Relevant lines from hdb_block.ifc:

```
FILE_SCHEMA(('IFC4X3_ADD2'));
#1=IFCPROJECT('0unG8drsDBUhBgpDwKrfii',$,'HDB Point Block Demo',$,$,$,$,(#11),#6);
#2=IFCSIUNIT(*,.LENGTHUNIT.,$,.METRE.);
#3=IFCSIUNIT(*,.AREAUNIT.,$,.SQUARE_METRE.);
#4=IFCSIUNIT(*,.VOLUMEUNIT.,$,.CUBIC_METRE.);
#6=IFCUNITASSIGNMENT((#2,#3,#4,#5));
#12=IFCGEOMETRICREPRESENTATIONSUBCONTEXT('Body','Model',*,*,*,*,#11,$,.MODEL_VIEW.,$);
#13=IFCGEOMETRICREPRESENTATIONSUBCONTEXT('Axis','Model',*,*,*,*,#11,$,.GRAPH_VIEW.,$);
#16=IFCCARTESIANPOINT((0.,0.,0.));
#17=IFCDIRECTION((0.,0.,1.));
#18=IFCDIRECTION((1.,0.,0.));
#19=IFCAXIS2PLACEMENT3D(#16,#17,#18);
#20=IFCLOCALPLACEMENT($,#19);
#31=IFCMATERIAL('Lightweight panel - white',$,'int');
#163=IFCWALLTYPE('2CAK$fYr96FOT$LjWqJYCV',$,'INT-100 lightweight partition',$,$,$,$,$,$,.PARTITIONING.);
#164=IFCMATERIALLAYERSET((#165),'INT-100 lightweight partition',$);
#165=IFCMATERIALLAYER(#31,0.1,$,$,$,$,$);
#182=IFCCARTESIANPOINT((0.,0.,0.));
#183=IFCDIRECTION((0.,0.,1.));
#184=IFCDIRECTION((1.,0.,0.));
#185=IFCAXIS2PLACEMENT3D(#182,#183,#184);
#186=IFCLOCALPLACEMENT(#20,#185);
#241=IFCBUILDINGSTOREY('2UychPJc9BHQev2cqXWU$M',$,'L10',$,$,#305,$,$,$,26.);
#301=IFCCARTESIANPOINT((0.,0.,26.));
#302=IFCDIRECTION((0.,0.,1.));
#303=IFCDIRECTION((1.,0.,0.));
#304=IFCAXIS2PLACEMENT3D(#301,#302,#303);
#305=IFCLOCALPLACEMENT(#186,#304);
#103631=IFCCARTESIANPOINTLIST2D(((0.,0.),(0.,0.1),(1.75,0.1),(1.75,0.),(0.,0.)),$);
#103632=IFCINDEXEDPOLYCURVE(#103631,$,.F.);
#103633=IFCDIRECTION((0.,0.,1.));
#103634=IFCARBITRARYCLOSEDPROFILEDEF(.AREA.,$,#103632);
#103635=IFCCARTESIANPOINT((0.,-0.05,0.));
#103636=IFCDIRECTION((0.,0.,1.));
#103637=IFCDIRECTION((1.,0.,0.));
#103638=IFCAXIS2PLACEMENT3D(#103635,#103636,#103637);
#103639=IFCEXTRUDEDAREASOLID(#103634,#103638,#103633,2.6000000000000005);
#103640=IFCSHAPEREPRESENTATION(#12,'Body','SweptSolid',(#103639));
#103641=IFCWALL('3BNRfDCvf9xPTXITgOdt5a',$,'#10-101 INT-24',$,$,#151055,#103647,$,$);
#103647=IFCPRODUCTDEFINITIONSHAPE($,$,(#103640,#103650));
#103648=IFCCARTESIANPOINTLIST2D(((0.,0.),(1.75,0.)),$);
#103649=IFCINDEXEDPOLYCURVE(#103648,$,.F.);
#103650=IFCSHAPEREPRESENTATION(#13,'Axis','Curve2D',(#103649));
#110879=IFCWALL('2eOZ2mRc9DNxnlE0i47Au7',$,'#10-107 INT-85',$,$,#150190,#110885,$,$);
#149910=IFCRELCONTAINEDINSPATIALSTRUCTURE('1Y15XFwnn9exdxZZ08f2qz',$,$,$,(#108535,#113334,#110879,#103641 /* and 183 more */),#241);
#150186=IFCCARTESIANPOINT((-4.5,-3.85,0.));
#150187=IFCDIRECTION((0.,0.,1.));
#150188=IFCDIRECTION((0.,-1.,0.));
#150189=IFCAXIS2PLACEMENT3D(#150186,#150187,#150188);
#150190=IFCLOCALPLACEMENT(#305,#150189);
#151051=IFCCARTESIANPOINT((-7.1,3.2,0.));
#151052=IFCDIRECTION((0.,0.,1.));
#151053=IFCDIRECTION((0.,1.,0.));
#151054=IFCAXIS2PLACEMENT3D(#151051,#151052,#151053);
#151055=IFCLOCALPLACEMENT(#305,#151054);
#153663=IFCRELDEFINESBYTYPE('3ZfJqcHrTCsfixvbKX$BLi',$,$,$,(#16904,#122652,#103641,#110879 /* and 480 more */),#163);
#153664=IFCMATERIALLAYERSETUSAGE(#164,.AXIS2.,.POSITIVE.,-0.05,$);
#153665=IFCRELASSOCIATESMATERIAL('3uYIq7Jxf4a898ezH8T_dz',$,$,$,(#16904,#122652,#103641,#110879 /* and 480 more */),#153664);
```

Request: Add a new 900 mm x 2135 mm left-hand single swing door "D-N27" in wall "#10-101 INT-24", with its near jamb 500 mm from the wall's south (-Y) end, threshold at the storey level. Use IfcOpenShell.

```python
import numpy as np
import ifcopenshell
import ifcopenshell.api.feature
import ifcopenshell.api.geometry
import ifcopenshell.api.root
import ifcopenshell.api.spatial
import ifcopenshell.geom
import ifcopenshell.util.element
import ifcopenshell.util.placement
import ifcopenshell.util.representation
import ifcopenshell.util.shape
import ifcopenshell.util.unit

model = ifcopenshell.open("hdb_block.ifc")
unit_scale = ifcopenshell.util.unit.calculate_unit_scale(model)
settings = ifcopenshell.geom.settings()


def volume(element):
    """Net volume in cubic metres, openings subtracted."""
    shape = ifcopenshell.geom.create_shape(settings, element)
    return ifcopenshell.util.shape.get_volume(shape.geometry)


wall = model.by_guid("3BNRfDCvf9xPTXITgOdt5a")
storey = ifcopenshell.util.element.get_container(wall, ifc_class="IfcBuildingStorey")
context = ifcopenshell.util.representation.get_context(model, "Model", "Body", "MODEL_VIEW")
before = volume(wall)

width, height, from_end, sill = 0.9, 2.135, 0.5, 0.0  # metres

# The wall runs along its own X axis, and the end named is its -X end.
wall_shape = ifcopenshell.geom.create_shape(settings, wall)
x, y, z = ifcopenshell.util.shape.get_vertices(wall_shape.geometry).T
start = x.min() + from_end
face, thickness = float(y.min()), float(y.max() - y.min())
wall_matrix = ifcopenshell.util.placement.get_local_placement(wall.ObjectPlacement)
level = ifcopenshell.util.placement.get_local_placement(storey.ObjectPlacement)[2, 3]


def in_wall(x, y):
    """Placement at x, y metres in the wall's axes, at sill height."""
    matrix = wall_matrix.copy()
    matrix[:, 3] = wall_matrix @ np.array([x / unit_scale, y / unit_scale, 0.0, 1.0])
    matrix[2, 3] = level + sill / unit_scale
    return matrix


# Opening: a box that overshoots both wall faces by 50 mm.
opening = ifcopenshell.api.root.create_entity(model, ifc_class="IfcOpeningElement", predefined_type="OPENING")
box = ifcopenshell.api.geometry.add_wall_representation(
    model, context=context, length=width, height=height, thickness=thickness + 0.1
)
ifcopenshell.api.geometry.assign_representation(model, product=opening, representation=box)
ifcopenshell.api.geometry.edit_object_placement(model, product=opening, matrix=in_wall(start, face - 0.05), is_si=False)
ifcopenshell.api.feature.add_feature(model, feature=opening, element=wall)

door = ifcopenshell.api.root.create_entity(model, ifc_class="IfcDoor", name="D-N27", predefined_type="DOOR")
door.OverallWidth, door.OverallHeight = width / unit_scale, height / unit_scale
door.OperationType = "SINGLE_SWING_LEFT"
body = ifcopenshell.api.geometry.add_door_representation(
    model,
    context=context,
    overall_width=door.OverallWidth,
    overall_height=door.OverallHeight,
    operation_type="SINGLE_SWING_LEFT",
    lining_properties={"LiningDepth": thickness / unit_scale, "ThresholdDepth": thickness / unit_scale},
)
ifcopenshell.api.geometry.assign_representation(model, product=door, representation=body)
ifcopenshell.api.spatial.assign_container(model, products=[door], relating_structure=storey)
ifcopenshell.api.feature.add_filling(model, opening=opening, element=door)

# The lining spans the wall, so the door starts at the wall face.
ifcopenshell.api.geometry.edit_object_placement(model, product=door, matrix=in_wall(start, face), is_si=False)

after = volume(wall)

print(f"wall volume {before:.3f} -> {after:.3f} m3")

model.write("hdb_block_rev.ifc")
```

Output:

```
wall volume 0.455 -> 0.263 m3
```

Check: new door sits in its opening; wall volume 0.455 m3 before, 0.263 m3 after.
